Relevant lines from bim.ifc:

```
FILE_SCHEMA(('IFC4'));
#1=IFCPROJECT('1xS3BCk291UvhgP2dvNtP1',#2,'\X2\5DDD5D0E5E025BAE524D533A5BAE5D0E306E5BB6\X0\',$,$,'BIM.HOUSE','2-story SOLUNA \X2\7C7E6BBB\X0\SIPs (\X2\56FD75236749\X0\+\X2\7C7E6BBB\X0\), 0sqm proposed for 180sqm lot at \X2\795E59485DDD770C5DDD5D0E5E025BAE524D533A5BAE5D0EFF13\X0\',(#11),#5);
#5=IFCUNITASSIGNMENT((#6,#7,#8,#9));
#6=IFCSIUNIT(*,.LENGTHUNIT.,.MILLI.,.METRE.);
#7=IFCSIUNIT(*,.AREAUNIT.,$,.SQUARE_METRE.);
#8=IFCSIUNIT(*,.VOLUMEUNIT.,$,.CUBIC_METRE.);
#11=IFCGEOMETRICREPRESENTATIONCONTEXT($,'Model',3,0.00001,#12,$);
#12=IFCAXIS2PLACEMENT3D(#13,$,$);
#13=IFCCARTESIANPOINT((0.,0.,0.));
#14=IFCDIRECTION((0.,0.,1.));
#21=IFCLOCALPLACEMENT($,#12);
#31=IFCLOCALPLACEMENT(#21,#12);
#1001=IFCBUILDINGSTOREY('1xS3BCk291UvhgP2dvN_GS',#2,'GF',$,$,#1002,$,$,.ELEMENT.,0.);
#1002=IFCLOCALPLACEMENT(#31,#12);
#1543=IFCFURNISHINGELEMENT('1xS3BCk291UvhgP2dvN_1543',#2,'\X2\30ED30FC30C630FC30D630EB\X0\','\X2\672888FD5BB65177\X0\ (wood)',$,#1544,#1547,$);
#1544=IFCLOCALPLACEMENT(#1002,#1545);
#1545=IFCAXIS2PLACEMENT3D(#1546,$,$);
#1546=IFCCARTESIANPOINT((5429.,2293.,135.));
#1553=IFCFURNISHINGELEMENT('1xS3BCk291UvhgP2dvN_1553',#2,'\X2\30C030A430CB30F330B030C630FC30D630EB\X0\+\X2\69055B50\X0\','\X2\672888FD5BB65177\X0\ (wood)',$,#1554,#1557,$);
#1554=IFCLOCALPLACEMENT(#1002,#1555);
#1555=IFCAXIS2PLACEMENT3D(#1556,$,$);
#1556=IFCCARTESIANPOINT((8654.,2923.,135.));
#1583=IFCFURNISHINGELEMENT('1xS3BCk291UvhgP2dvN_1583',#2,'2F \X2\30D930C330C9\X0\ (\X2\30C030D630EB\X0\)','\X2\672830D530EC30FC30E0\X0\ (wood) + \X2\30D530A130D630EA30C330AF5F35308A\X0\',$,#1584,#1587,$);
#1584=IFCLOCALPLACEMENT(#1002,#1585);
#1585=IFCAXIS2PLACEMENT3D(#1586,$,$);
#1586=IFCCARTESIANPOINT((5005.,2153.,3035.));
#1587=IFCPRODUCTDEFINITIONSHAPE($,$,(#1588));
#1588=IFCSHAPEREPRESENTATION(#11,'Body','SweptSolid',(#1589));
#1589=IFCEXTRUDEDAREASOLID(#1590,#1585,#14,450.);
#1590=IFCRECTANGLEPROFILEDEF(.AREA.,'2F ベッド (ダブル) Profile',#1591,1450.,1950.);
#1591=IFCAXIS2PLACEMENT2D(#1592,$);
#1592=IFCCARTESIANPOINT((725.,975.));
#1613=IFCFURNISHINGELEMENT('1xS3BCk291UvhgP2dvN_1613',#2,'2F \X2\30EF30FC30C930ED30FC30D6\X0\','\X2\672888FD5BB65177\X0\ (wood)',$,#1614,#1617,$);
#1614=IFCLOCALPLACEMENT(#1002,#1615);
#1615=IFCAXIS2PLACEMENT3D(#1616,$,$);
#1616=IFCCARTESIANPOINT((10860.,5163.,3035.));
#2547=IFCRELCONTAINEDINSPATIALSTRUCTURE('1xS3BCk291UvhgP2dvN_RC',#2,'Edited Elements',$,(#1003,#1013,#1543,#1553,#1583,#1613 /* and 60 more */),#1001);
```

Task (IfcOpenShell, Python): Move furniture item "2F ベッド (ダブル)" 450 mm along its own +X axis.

```python
import ifcopenshell
import ifcopenshell.api.geometry
import ifcopenshell.util.placement
import ifcopenshell.util.unit

model = ifcopenshell.open("bim.ifc")
unit_scale = ifcopenshell.util.unit.calculate_unit_scale(model)

item = model.by_id(1583)
matrix = ifcopenshell.util.placement.get_local_placement(item.ObjectPlacement)
matrix[:3, 3] += matrix[:3, 0] * 0.45 / unit_scale
ifcopenshell.api.geometry.edit_object_placement(model, product=item, matrix=matrix, is_si=False)

print(ifcopenshell.util.placement.get_local_placement(item.ObjectPlacement).round(3) + 0.0)

model.write("bim-out.ifc")
```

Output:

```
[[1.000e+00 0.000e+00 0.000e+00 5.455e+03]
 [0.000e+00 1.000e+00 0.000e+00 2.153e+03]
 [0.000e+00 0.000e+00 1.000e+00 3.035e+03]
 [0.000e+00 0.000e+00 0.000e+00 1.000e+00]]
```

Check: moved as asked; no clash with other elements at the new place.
